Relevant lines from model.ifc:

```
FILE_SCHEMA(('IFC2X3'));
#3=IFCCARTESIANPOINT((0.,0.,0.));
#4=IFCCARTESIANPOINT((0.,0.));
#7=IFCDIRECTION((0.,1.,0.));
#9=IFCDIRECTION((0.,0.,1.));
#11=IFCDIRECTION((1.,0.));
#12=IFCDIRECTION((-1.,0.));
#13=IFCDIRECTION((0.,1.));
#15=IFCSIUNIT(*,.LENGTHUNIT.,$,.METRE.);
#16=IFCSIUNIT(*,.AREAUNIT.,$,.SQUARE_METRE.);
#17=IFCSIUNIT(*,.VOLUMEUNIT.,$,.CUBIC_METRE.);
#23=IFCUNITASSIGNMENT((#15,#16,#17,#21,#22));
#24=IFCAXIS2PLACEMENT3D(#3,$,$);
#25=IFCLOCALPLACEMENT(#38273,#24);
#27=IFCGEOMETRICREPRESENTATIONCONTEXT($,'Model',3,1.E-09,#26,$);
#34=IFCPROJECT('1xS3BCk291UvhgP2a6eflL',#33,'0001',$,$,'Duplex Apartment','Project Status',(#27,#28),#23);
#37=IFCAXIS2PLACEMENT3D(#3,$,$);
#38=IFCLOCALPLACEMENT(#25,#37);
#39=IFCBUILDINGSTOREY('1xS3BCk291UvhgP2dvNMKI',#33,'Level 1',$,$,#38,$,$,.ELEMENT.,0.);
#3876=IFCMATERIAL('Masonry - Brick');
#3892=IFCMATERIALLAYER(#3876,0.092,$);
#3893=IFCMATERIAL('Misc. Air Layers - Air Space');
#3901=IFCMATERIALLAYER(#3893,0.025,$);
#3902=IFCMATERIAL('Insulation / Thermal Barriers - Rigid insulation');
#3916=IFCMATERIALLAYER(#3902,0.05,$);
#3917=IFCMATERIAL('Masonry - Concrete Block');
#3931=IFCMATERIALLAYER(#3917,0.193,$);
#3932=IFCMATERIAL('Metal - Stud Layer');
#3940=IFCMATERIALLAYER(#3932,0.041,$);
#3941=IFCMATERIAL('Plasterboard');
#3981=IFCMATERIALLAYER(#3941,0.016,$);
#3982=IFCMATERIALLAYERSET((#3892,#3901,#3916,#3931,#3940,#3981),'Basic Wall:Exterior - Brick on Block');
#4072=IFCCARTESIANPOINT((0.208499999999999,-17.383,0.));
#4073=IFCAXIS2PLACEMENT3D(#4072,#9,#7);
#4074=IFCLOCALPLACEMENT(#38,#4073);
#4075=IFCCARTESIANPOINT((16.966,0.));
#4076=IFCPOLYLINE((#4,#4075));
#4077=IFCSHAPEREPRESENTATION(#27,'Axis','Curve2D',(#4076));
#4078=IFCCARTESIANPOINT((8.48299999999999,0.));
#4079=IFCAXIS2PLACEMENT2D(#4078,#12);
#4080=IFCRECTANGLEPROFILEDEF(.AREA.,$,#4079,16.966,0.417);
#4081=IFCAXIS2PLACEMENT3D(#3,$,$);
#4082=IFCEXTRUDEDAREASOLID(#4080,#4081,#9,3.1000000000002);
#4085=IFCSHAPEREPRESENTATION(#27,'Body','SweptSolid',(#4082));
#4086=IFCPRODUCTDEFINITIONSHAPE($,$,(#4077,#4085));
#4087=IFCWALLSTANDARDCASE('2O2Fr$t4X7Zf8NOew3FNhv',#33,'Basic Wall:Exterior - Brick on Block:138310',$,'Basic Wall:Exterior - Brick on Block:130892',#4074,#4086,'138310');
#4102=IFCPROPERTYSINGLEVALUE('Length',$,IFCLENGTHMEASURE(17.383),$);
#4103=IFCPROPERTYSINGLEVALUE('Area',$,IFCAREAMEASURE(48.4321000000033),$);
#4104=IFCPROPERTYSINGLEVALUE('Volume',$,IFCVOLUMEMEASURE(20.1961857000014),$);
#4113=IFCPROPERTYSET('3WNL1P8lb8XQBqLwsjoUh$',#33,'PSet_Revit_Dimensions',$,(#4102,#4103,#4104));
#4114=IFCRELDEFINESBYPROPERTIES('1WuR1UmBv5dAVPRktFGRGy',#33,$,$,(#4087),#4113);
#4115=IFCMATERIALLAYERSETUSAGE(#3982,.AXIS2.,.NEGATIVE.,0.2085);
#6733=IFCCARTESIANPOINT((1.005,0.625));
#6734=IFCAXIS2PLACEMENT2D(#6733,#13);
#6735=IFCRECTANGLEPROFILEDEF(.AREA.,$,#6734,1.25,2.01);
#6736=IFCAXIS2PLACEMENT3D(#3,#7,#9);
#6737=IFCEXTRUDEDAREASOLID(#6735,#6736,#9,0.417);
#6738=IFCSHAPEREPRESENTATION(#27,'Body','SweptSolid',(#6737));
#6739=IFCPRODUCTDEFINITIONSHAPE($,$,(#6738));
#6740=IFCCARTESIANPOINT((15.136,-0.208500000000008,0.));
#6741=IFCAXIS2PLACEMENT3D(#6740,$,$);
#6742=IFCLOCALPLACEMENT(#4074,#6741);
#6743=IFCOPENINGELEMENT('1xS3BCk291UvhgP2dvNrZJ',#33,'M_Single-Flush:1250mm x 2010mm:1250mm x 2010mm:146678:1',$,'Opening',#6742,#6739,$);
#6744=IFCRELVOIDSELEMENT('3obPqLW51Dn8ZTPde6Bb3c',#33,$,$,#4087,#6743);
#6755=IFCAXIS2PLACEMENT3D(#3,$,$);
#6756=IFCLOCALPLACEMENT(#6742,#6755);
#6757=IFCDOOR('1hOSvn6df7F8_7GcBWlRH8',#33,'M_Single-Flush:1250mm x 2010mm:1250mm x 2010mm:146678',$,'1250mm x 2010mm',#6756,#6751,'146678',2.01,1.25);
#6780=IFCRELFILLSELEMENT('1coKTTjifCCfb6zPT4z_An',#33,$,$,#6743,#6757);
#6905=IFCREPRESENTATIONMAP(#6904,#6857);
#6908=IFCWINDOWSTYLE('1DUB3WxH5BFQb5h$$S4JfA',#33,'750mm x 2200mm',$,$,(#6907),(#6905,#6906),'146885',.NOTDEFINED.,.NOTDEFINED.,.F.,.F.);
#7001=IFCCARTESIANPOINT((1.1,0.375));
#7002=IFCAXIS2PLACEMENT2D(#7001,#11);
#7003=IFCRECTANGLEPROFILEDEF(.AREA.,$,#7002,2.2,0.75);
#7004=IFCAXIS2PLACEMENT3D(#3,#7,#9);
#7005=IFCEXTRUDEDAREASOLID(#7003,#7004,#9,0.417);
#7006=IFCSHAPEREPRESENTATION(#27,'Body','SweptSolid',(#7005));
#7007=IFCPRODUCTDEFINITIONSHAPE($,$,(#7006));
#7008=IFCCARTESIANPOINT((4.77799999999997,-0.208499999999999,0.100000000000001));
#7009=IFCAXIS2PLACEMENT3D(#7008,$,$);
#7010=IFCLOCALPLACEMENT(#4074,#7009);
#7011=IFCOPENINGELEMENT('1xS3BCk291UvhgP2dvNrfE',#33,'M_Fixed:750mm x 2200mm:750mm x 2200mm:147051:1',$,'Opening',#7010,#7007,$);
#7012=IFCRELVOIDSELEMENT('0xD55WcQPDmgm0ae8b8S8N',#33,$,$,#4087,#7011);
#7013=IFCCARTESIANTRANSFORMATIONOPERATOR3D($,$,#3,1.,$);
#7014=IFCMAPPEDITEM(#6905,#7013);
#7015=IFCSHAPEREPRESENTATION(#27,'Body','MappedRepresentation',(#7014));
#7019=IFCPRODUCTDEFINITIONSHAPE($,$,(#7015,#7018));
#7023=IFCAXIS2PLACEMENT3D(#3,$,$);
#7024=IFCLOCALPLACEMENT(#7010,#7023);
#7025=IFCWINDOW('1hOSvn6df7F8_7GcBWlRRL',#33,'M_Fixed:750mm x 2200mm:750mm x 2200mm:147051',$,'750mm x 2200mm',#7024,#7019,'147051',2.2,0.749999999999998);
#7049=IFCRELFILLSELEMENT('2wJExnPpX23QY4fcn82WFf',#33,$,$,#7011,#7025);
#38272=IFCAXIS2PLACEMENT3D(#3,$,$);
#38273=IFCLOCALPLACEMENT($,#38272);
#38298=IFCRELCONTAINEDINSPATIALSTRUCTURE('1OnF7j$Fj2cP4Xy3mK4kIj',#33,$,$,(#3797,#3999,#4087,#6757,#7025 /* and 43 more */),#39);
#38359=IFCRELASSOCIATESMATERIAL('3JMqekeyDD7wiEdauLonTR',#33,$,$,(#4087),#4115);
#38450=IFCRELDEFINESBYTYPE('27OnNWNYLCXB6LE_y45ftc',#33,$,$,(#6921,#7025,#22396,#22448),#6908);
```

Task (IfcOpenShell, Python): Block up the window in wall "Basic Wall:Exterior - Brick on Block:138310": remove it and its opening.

```python
import ifcopenshell
import ifcopenshell.api.feature
import ifcopenshell.api.pset
import ifcopenshell.api.root
import ifcopenshell.geom
import ifcopenshell.util.element
import ifcopenshell.util.shape
import ifcopenshell.util.unit

model = ifcopenshell.open("model.ifc")
area_scale = ifcopenshell.util.unit.calculate_unit_scale(model, "AREAUNIT")
volume_scale = ifcopenshell.util.unit.calculate_unit_scale(model, "VOLUMEUNIT")
settings = ifcopenshell.geom.settings()


def volume(element):
    """Net volume in cubic metres, openings subtracted."""
    shape = ifcopenshell.geom.create_shape(settings, element)
    return ifcopenshell.util.shape.get_volume(shape.geometry)


window = model.by_guid("1hOSvn6df7F8_7GcBWlRRL")
opening = window.FillsVoids[0].RelatingOpeningElement
wall = opening.VoidsElements[0].RelatingBuildingElement
before = volume(wall)

ifcopenshell.api.root.remove_product(model, product=window)
ifcopenshell.api.feature.remove_feature(model, feature=opening)

after = volume(wall)
thickness = 0.417  # wall thickness in metres

# Update the wall's stored quantities.
pset = model.by_id(ifcopenshell.util.element.get_pset(wall, "PSet_Revit_Dimensions", should_inherit=False)["id"])
ifcopenshell.api.pset.edit_pset(model, pset=pset, properties={
    "Area": model.create_entity("IfcAreaMeasure", after / thickness / area_scale),
    "Volume": model.create_entity("IfcVolumeMeasure", after / volume_scale),
})

print(f"wall volume {before:.3f} -> {after:.3f} m3")

model.write("model_edited.ifc")
```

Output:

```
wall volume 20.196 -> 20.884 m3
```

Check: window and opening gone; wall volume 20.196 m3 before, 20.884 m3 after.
